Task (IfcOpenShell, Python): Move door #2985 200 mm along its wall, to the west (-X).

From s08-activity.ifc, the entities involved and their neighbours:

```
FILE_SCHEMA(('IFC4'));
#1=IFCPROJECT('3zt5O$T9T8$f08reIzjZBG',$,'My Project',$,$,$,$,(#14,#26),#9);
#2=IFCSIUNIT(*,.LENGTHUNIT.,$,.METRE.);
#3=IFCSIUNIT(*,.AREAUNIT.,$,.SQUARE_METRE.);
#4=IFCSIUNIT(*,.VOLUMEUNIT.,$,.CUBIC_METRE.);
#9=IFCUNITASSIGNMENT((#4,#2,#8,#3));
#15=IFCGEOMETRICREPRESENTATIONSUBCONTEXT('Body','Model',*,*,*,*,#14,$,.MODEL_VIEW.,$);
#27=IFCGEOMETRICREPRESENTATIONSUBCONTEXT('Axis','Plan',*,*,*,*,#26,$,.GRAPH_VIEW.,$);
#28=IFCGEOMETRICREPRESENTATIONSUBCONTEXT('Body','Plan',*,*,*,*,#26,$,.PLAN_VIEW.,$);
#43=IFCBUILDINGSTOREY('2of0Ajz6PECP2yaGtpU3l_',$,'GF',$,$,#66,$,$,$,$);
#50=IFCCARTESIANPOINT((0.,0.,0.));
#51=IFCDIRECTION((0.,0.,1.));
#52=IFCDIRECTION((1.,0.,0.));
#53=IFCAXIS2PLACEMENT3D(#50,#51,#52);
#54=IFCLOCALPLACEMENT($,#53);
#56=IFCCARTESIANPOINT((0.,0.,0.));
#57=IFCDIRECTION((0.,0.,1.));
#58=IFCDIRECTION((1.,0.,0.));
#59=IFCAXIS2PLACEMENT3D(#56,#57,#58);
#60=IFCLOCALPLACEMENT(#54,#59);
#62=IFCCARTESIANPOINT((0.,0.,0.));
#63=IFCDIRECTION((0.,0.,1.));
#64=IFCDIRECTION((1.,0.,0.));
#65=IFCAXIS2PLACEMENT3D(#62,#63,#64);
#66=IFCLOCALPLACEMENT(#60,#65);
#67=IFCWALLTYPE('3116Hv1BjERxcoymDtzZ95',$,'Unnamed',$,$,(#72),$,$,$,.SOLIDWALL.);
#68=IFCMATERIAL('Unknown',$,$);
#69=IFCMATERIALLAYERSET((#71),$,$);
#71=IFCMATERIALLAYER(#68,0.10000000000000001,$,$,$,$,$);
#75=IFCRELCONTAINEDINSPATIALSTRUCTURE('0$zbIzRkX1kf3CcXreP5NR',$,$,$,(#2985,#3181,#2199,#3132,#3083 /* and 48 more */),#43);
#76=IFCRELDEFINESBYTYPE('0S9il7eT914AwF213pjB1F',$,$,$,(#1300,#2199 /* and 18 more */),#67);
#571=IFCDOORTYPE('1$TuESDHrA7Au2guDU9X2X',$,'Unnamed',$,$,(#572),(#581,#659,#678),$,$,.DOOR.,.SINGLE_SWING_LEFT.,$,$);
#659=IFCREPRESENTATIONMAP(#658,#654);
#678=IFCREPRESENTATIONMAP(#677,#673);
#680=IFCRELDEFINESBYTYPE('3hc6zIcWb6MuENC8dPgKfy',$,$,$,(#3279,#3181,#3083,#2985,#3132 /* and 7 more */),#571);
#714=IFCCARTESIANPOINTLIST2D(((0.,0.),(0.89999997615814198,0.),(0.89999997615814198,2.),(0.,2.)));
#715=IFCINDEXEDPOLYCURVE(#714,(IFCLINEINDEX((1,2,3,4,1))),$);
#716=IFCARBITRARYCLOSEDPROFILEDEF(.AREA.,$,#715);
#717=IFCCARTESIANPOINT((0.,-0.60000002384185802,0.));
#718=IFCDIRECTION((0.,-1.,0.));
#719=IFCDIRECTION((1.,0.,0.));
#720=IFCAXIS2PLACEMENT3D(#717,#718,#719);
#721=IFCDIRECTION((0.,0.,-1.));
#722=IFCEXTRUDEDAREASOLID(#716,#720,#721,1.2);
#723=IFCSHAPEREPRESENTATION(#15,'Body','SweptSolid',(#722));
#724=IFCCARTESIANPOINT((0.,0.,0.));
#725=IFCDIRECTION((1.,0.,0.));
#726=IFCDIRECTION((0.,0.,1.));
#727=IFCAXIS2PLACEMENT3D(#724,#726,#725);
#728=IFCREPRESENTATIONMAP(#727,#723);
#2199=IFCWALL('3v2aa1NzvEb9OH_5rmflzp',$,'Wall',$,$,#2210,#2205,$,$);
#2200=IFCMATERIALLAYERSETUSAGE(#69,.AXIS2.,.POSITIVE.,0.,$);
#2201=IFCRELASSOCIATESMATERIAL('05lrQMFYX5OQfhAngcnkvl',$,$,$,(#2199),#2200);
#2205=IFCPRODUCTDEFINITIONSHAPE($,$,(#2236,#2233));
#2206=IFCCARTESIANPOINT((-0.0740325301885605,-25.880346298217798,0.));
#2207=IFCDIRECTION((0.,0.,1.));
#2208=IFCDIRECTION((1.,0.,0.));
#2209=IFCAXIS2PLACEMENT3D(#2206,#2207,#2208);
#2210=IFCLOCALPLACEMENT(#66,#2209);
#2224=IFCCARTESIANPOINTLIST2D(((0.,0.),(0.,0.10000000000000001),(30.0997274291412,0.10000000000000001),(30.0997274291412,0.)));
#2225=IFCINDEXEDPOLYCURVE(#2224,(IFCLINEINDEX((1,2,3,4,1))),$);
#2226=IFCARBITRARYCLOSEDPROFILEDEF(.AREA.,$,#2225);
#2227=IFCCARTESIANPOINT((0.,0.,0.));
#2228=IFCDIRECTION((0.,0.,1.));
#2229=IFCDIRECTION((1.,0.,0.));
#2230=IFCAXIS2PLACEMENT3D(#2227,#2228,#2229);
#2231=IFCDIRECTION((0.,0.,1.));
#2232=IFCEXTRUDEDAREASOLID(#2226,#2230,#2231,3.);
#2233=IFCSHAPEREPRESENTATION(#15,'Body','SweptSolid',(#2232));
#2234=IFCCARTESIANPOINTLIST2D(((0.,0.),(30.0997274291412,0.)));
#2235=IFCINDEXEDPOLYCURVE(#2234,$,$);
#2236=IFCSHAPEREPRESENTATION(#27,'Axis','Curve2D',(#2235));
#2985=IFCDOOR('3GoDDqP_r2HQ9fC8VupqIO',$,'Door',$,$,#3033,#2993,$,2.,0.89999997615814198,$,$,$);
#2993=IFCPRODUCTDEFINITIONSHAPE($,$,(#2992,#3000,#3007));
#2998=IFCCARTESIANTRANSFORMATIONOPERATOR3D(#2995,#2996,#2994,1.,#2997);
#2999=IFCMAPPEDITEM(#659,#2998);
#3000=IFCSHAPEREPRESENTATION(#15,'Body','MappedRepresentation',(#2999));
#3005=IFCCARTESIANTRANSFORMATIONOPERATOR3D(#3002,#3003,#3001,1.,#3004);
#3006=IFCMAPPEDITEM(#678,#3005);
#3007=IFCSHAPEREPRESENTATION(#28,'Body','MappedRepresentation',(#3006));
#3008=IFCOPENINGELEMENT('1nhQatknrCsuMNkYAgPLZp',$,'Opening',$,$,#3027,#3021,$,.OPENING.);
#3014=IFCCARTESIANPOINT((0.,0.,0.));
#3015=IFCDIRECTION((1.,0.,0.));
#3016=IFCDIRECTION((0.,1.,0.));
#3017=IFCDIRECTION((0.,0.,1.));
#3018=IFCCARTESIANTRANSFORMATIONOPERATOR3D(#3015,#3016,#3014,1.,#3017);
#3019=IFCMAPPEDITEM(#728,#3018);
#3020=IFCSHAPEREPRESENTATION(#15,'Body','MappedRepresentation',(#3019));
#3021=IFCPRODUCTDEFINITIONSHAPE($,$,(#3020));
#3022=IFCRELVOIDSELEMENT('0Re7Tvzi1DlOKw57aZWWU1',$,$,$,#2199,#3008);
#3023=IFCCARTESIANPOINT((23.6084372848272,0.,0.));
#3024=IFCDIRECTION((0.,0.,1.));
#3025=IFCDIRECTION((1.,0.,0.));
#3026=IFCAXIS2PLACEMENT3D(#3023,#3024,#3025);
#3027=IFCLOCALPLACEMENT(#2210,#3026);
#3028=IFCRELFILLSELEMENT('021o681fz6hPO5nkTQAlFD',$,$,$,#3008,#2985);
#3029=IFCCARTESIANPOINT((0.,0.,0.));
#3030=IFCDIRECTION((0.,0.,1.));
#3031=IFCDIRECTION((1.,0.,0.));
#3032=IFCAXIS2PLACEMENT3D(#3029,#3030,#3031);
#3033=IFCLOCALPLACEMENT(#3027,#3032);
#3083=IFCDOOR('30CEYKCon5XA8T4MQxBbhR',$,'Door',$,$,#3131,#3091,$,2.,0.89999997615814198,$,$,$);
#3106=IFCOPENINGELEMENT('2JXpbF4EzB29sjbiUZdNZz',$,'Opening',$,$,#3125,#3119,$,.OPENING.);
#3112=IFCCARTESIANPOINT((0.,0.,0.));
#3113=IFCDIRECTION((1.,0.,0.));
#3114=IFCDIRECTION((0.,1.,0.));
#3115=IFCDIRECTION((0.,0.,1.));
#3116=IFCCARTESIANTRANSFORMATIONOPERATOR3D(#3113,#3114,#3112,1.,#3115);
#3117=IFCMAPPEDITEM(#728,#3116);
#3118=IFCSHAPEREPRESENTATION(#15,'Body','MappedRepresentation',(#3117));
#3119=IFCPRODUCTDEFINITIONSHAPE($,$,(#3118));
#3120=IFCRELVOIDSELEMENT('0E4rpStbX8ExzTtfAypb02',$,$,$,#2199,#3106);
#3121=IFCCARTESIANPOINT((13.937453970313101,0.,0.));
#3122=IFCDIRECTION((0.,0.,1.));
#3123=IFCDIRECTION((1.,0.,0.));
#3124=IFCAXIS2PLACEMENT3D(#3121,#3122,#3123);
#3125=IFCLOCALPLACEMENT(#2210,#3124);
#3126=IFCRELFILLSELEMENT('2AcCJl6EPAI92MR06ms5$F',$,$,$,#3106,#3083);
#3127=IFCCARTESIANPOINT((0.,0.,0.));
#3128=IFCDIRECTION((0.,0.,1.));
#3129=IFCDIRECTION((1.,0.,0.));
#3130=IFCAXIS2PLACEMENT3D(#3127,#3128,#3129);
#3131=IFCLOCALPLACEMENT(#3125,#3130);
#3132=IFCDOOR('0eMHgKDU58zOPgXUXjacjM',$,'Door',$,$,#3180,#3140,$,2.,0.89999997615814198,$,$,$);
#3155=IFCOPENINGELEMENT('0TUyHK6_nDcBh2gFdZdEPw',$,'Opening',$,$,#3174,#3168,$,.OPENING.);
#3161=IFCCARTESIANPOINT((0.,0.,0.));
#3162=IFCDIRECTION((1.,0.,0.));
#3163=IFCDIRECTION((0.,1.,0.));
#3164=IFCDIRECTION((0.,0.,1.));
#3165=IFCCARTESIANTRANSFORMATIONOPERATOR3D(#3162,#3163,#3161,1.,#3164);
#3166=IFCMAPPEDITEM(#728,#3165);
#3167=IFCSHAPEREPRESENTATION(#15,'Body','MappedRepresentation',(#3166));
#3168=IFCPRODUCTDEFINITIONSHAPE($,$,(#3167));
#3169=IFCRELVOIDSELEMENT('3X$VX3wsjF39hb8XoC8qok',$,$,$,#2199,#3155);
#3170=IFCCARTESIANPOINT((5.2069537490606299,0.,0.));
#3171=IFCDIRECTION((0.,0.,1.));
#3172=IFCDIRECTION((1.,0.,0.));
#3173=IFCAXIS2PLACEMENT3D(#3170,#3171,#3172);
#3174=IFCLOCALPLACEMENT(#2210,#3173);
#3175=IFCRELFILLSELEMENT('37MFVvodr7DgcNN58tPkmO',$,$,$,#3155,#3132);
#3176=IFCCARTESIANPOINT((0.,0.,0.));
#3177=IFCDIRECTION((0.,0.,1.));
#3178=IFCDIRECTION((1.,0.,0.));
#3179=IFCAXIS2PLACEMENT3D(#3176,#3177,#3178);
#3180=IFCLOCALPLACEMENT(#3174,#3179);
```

```python
import ifcopenshell
import ifcopenshell.api.geometry
import ifcopenshell.util.placement

model = ifcopenshell.open("s08-activity.ifc")

door = model.by_guid("3GoDDqP_r2HQ9fC8VupqIO")
opening = door.FillsVoids[0].RelatingOpeningElement
wall = opening.VoidsElements[0].RelatingBuildingElement

wall_matrix = ifcopenshell.util.placement.get_local_placement(wall.ObjectPlacement)
shift = wall_matrix[:3, 0] * -0.2
before = ifcopenshell.util.placement.get_local_placement(door.ObjectPlacement)[:3, 3].copy()

# The door is placed relative to its opening, so it follows when the opening moves.
matrix = ifcopenshell.util.placement.get_local_placement(opening.ObjectPlacement)
matrix[:3, 3] += shift
ifcopenshell.api.geometry.edit_object_placement(
    model, product=opening, matrix=matrix, is_si=False, should_transform_children=True
)

after = ifcopenshell.util.placement.get_local_placement(door.ObjectPlacement)[:3, 3]
print("door moved by", (after - before).round(3) + 0.0)

model.write("s08-activity_edited.ifc")
```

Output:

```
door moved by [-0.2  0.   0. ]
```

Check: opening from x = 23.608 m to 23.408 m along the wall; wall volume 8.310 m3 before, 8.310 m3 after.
